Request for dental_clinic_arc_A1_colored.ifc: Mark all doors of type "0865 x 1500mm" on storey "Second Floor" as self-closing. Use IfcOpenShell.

First a look at what the model holds.

```python
import ifcopenshell
import ifcopenshell.util.element

model = ifcopenshell.open("dental_clinic_arc_A1_colored.ifc")
print(model.schema)
storey = next(s for s in model.by_type("IfcBuildingStorey") if s.Name == "Second Floor")
doors = [e for e in ifcopenshell.util.element.get_decomposition(storey) if e.is_a("IfcDoor")]
seen = {}
for e in doors:
    element_type = ifcopenshell.util.element.get_type(e)
    key = (element_type.Name if element_type != e and element_type else None, ifcopenshell.util.element.get_pset(e, "Pset_DoorCommon", "SelfClosing"))
    seen[key] = seen.get(key, 0) + 1
for (name, value), count in sorted(seen.items(), key=str):
    print(count, "x", name, "|", value)
```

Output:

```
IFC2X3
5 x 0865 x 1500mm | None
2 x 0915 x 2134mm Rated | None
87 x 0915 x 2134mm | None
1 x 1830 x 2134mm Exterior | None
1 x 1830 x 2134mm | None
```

```python
import ifcopenshell
import ifcopenshell.api.pset
import ifcopenshell.util.element

model = ifcopenshell.open("dental_clinic_arc_A1_colored.ifc")

storey = next(s for s in model.by_type("IfcBuildingStorey") if s.Name == "Second Floor")
doors = [e for e in ifcopenshell.util.element.get_decomposition(storey) if e.is_a("IfcDoor")]

count = 0
for e in doors:
    element_type = ifcopenshell.util.element.get_type(e)
    if element_type in (None, e) or element_type.Name != "0865 x 1500mm":
        continue
    # add_pset returns the element's existing set when there is one.
    pset = ifcopenshell.api.pset.add_pset(model, product=e, name="Pset_DoorCommon")
    ifcopenshell.api.pset.edit_pset(model, pset=pset, properties={"SelfClosing": True})
    count += 1

print(count, "doors updated")

model.write("dental_clinic_arc_A1_colored-out.ifc")
```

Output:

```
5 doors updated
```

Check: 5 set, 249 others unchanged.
